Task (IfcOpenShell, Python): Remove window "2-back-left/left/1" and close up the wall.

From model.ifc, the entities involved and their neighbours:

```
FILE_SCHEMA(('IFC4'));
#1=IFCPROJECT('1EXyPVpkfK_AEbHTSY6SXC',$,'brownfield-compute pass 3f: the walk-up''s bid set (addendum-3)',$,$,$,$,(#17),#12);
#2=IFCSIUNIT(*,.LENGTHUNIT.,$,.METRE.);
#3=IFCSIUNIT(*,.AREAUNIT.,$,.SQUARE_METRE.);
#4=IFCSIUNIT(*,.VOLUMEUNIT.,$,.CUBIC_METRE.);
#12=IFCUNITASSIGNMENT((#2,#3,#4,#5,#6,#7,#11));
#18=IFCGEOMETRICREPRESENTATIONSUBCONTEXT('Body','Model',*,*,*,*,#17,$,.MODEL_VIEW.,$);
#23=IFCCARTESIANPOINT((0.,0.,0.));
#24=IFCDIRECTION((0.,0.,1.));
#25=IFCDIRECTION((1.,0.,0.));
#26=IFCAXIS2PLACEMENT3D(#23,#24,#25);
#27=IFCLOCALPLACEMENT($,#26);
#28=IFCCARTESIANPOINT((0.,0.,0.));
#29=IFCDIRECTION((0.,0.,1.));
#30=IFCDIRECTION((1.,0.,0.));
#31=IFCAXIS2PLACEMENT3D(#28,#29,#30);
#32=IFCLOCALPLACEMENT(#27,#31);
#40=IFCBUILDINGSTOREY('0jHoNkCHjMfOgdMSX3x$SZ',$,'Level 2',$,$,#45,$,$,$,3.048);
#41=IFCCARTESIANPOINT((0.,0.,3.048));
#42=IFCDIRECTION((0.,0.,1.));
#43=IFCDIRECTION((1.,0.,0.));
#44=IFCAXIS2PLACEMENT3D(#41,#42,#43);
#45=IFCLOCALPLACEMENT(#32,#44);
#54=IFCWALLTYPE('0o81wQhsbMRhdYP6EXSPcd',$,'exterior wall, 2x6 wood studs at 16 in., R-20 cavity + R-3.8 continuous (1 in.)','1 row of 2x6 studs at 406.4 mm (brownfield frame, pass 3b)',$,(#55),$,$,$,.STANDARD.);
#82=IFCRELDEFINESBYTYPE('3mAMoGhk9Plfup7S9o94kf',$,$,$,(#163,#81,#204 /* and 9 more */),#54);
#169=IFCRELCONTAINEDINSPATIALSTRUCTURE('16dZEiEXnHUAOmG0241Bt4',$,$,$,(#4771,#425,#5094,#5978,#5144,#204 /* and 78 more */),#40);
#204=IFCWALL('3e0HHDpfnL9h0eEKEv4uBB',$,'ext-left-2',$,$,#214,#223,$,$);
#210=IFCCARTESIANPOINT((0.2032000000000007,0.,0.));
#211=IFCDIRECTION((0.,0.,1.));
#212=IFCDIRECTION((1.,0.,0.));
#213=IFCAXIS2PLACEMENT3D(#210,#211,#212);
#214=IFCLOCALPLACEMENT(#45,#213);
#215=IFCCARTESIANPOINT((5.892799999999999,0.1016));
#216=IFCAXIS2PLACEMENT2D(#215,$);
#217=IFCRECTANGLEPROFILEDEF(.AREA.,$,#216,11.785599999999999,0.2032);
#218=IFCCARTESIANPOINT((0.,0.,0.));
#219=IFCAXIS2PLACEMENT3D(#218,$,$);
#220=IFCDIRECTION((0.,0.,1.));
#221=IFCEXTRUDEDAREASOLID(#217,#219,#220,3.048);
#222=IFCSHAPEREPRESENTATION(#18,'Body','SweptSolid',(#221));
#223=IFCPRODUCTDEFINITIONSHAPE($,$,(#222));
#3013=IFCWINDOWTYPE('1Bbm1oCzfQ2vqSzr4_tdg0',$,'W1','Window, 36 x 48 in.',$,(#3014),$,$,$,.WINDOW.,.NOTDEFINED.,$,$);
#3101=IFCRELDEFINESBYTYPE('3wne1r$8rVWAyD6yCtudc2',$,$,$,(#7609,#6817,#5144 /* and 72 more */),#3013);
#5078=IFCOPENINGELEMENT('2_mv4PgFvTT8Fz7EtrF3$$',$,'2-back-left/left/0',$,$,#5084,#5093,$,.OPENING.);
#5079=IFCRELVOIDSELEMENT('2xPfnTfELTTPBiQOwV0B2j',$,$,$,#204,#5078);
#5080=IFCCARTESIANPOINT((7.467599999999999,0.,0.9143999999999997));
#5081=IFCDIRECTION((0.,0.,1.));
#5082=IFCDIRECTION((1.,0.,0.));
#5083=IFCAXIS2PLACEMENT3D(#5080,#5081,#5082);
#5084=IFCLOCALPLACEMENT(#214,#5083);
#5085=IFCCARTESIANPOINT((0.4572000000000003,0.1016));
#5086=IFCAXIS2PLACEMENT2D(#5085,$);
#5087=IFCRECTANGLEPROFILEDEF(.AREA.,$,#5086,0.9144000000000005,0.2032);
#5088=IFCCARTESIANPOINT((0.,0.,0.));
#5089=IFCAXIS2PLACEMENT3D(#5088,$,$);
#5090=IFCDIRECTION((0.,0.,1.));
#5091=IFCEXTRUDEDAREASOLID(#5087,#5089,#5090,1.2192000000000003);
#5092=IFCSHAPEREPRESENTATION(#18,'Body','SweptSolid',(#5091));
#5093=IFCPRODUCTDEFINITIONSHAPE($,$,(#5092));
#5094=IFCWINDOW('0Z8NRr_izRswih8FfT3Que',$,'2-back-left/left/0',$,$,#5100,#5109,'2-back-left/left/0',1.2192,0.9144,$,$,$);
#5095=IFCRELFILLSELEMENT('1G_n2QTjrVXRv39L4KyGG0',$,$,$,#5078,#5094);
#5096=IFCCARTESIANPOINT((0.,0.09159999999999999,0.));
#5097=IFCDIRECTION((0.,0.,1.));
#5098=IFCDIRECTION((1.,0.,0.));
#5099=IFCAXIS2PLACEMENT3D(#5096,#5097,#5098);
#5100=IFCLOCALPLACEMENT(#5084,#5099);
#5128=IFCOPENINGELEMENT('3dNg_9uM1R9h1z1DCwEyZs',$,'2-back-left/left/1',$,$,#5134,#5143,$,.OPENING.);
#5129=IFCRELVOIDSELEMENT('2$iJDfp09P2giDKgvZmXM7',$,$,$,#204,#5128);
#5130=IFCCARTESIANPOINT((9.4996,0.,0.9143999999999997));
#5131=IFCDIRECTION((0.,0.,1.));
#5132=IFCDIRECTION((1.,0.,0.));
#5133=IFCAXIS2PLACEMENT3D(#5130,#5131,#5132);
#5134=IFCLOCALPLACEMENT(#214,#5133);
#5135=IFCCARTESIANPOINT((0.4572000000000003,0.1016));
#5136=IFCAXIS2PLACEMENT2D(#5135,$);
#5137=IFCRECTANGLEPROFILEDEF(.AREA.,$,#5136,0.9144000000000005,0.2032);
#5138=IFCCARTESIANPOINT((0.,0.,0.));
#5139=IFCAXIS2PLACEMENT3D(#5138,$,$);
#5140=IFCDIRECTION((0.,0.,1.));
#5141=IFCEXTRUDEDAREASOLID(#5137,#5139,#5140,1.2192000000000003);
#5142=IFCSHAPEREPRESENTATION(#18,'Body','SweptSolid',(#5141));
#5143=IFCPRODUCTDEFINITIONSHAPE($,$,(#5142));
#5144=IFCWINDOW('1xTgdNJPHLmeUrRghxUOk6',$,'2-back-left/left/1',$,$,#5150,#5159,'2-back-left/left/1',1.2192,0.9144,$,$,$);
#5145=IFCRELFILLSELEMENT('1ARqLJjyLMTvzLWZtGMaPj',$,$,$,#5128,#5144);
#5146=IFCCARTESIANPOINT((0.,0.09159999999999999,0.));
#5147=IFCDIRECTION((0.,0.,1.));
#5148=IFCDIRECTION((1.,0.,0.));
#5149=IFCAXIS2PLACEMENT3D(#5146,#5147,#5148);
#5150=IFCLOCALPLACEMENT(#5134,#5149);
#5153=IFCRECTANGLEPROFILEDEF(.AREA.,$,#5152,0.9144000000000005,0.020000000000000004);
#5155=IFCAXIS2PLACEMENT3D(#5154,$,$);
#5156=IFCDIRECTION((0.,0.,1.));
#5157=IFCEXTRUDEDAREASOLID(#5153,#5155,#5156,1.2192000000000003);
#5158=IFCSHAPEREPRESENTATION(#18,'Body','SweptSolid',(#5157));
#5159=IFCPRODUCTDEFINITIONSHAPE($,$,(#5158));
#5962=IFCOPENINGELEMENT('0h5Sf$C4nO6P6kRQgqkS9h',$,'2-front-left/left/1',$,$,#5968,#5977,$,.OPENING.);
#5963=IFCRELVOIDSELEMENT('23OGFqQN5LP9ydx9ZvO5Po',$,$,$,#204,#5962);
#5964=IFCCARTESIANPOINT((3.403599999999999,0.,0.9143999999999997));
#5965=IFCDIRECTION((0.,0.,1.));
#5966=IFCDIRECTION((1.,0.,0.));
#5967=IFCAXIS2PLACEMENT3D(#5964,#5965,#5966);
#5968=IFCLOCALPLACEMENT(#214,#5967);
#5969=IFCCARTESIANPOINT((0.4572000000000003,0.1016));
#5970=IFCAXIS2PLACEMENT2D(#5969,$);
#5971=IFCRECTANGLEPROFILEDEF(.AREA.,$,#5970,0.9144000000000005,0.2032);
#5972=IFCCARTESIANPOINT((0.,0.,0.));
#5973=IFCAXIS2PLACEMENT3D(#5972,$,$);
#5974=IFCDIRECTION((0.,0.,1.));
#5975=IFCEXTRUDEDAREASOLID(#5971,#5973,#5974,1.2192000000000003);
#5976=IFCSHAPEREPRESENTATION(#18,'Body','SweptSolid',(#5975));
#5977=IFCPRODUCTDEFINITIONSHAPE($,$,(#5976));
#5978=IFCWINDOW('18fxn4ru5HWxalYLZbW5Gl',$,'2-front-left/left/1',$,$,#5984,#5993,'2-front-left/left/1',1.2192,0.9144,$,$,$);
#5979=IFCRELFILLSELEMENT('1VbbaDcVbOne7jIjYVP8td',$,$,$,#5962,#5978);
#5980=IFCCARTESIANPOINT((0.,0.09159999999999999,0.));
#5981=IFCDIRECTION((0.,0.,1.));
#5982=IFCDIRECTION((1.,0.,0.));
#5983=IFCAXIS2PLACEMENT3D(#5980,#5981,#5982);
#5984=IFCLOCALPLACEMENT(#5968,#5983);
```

```python
import ifcopenshell
import ifcopenshell.api.feature
import ifcopenshell.api.root
import ifcopenshell.geom
import ifcopenshell.util.shape

model = ifcopenshell.open("model.ifc")
settings = ifcopenshell.geom.settings()


def volume(element):
    """Net volume in cubic metres, openings subtracted."""
    shape = ifcopenshell.geom.create_shape(settings, element)
    return ifcopenshell.util.shape.get_volume(shape.geometry)


window = model.by_guid("1xTgdNJPHLmeUrRghxUOk6")
opening = window.FillsVoids[0].RelatingOpeningElement
wall = opening.VoidsElements[0].RelatingBuildingElement
before = volume(wall)

ifcopenshell.api.root.remove_product(model, product=window)
ifcopenshell.api.feature.remove_feature(model, feature=opening)

after = volume(wall)

print(f"wall volume {before:.3f} -> {after:.3f} m3")

model.write("model_updated.ifc")
```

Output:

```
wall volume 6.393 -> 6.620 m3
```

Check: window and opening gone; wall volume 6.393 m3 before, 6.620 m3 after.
